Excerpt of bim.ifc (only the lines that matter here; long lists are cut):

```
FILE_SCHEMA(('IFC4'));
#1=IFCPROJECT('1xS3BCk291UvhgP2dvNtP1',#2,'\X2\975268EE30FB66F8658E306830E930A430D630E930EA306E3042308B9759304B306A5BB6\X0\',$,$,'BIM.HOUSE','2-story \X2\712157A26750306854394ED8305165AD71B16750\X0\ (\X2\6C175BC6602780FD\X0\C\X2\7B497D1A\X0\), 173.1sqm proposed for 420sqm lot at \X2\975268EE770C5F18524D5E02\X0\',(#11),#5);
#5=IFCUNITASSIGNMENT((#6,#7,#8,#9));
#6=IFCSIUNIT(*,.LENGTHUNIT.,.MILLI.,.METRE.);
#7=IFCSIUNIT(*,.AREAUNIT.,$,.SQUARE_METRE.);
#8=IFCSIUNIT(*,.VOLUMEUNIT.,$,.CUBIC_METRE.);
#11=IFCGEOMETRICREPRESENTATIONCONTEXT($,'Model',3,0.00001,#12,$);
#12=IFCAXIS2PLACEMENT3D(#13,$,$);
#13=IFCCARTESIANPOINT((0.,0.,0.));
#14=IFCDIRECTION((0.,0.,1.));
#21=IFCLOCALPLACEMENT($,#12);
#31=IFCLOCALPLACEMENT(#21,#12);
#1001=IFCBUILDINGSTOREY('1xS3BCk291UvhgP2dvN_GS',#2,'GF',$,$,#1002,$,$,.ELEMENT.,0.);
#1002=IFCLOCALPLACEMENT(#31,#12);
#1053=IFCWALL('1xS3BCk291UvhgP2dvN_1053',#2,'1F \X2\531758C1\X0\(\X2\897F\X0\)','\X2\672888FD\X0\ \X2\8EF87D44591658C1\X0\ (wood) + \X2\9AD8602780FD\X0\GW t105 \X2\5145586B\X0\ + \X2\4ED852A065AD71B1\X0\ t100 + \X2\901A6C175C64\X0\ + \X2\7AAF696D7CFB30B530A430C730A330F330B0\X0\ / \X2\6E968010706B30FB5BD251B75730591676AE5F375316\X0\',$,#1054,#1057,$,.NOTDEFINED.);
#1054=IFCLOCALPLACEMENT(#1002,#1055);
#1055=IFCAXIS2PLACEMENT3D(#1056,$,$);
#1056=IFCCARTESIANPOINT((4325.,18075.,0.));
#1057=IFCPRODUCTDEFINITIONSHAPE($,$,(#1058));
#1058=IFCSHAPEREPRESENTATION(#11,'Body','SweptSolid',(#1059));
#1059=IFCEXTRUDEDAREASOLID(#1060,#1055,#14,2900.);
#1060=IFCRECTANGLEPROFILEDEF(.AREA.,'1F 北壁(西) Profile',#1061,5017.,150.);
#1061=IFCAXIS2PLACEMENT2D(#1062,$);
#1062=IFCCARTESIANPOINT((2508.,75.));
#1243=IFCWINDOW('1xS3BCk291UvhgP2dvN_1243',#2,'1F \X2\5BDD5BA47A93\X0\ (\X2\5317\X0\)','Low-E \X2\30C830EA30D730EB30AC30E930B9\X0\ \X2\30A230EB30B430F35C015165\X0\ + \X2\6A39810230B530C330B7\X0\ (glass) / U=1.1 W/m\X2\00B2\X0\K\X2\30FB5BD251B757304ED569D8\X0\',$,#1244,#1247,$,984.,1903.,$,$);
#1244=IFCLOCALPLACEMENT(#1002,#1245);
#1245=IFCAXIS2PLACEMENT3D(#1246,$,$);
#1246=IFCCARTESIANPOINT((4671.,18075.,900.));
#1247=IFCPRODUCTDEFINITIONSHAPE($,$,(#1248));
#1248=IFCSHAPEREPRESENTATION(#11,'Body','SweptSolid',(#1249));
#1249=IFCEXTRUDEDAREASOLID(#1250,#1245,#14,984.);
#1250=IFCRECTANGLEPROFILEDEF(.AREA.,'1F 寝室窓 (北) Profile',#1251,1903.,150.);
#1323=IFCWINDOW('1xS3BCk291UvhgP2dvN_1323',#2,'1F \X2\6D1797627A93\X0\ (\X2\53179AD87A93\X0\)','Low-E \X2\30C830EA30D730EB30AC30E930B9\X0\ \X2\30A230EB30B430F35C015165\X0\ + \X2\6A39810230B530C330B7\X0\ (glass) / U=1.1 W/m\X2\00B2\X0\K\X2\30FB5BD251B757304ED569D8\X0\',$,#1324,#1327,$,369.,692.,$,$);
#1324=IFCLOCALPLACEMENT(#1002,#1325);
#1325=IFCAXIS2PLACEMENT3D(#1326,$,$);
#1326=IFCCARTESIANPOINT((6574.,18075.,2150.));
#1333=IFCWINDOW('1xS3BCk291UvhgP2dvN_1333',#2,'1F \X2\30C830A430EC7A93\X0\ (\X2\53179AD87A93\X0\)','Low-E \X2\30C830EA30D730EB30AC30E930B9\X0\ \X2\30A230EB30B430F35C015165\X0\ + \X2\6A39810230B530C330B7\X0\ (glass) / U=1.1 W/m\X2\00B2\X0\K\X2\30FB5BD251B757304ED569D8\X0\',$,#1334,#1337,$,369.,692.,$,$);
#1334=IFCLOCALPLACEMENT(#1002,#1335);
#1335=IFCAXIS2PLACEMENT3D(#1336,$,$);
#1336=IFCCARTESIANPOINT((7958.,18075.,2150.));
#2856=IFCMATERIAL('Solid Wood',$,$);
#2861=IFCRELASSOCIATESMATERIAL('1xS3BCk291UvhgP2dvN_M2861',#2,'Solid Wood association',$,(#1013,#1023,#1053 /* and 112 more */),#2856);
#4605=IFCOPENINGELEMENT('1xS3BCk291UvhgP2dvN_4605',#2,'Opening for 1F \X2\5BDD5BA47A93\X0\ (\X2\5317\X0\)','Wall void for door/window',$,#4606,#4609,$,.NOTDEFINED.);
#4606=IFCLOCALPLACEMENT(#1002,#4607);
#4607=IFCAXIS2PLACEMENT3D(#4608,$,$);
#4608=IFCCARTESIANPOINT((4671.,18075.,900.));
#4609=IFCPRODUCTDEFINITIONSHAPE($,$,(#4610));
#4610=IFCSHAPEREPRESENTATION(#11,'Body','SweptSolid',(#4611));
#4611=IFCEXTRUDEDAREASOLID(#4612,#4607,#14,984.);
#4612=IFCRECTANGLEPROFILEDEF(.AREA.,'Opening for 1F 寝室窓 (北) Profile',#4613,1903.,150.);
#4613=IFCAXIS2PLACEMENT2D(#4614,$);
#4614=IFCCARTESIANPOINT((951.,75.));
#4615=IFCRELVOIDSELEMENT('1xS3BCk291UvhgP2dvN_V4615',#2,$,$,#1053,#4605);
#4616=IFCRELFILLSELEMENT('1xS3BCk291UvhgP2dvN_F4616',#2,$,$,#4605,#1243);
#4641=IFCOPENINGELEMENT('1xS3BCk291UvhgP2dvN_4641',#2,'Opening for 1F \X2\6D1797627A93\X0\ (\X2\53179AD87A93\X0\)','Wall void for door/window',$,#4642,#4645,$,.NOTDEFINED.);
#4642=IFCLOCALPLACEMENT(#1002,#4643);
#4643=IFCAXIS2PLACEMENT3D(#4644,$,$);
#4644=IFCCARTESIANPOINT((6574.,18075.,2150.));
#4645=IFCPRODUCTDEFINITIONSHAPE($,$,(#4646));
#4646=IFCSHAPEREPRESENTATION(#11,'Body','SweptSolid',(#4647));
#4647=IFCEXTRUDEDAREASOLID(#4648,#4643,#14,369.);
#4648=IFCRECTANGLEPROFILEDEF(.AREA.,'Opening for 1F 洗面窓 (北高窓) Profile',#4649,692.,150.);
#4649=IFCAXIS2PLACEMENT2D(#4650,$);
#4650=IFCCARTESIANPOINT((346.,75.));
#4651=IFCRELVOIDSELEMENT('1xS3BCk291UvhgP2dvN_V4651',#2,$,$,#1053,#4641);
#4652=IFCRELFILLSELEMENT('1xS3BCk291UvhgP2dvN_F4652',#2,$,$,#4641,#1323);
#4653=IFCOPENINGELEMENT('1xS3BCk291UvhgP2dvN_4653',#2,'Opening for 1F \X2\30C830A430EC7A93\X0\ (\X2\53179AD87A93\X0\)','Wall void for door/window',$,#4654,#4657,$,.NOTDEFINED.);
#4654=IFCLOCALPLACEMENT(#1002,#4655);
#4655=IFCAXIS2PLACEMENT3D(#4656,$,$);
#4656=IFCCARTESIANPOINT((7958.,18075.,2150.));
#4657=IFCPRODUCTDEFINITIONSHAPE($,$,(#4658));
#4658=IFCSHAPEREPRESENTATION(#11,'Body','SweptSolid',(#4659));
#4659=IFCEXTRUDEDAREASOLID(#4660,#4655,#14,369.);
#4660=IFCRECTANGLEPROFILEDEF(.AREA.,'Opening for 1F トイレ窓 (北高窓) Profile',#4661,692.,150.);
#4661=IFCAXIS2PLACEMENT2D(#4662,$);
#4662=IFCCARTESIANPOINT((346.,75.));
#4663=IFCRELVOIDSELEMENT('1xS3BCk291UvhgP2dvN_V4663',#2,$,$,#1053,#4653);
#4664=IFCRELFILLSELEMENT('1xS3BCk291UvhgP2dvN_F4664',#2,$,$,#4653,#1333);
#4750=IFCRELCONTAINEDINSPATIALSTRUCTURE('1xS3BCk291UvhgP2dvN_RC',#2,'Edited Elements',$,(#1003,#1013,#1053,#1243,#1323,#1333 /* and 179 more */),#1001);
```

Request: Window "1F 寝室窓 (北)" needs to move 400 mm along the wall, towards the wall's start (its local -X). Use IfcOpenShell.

```python
import ifcopenshell
import ifcopenshell.api.geometry
import ifcopenshell.util.placement
import ifcopenshell.util.unit

model = ifcopenshell.open("bim.ifc")
unit_scale = ifcopenshell.util.unit.calculate_unit_scale(model)

window = model.by_guid("1xS3BCk291UvhgP2dvN_1243")
opening = window.FillsVoids[0].RelatingOpeningElement
wall = opening.VoidsElements[0].RelatingBuildingElement

wall_matrix = ifcopenshell.util.placement.get_local_placement(wall.ObjectPlacement)
shift = wall_matrix[:3, 0] * -0.4 / unit_scale
before = ifcopenshell.util.placement.get_local_placement(window.ObjectPlacement)[:3, 3].copy()

# The window is not placed relative to its opening, so move both.
for product in (opening, window):
    matrix = ifcopenshell.util.placement.get_local_placement(product.ObjectPlacement)
    matrix[:3, 3] += shift
    ifcopenshell.api.geometry.edit_object_placement(model, product=product, matrix=matrix, is_si=False)

after = ifcopenshell.util.placement.get_local_placement(window.ObjectPlacement)[:3, 3]
print("window moved by", (after - before).round(3) + 0.0)

model.write("bim_v2.ifc")
```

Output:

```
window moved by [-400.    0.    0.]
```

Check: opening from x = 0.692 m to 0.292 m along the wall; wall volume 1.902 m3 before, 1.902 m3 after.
